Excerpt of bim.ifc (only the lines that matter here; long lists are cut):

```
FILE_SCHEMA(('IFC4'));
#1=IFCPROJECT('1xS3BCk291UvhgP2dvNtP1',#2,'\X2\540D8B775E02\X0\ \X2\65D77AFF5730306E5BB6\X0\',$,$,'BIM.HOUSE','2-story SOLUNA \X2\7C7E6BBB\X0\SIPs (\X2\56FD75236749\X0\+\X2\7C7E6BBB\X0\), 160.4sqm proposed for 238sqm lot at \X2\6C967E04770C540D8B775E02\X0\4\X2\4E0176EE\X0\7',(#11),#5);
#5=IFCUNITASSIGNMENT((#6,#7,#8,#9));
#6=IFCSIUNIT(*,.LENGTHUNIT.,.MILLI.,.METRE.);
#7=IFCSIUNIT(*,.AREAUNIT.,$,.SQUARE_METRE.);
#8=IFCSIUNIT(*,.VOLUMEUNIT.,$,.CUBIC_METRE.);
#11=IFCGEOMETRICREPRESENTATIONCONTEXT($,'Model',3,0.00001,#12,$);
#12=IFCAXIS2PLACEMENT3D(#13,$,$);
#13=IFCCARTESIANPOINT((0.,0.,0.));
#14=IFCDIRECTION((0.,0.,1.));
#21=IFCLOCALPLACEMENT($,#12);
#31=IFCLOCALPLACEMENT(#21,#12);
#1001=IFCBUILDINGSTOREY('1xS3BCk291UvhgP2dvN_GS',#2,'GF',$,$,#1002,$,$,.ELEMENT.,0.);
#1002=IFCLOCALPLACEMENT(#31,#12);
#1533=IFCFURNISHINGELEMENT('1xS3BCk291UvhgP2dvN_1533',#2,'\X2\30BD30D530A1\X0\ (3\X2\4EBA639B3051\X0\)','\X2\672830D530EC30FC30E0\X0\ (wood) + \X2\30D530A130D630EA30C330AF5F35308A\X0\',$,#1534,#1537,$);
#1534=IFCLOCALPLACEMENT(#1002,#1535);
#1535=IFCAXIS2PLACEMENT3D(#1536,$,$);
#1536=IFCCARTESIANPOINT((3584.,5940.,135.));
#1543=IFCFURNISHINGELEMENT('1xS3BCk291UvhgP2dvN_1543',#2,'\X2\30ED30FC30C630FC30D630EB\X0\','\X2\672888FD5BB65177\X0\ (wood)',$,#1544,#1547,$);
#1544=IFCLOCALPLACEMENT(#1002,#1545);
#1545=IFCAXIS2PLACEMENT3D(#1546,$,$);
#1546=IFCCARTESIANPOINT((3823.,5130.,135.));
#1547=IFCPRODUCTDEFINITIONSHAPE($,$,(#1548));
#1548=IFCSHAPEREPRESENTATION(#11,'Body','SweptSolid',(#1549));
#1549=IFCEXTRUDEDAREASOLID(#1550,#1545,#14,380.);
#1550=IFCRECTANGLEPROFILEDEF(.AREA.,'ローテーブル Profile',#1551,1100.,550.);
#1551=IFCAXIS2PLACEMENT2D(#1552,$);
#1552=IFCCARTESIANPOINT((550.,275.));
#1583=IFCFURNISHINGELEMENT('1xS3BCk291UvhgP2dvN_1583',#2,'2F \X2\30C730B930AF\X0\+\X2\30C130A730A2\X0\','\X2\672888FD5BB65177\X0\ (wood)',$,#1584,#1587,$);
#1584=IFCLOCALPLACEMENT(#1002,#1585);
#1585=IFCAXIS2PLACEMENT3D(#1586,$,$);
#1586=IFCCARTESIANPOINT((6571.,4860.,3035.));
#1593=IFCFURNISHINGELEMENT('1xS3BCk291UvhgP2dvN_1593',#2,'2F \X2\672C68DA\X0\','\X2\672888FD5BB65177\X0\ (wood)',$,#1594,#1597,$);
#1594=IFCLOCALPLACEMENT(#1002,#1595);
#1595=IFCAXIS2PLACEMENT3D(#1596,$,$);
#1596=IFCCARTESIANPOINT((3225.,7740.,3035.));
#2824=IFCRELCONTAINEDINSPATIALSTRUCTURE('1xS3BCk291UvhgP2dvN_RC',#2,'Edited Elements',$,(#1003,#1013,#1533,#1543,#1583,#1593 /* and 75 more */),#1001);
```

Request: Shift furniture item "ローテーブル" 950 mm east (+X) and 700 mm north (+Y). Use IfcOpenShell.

```python
import ifcopenshell
import ifcopenshell.api.geometry
import ifcopenshell.util.placement
import ifcopenshell.util.unit

model = ifcopenshell.open("bim.ifc")
unit_scale = ifcopenshell.util.unit.calculate_unit_scale(model)

item = model.by_guid("1xS3BCk291UvhgP2dvN_1543")
matrix = ifcopenshell.util.placement.get_local_placement(item.ObjectPlacement)
matrix[0, 3] += 0.95 / unit_scale
matrix[1, 3] += 0.7 / unit_scale
ifcopenshell.api.geometry.edit_object_placement(model, product=item, matrix=matrix, is_si=False)

print(ifcopenshell.util.placement.get_local_placement(item.ObjectPlacement).round(3) + 0.0)

model.write("bim_v2.ifc")
```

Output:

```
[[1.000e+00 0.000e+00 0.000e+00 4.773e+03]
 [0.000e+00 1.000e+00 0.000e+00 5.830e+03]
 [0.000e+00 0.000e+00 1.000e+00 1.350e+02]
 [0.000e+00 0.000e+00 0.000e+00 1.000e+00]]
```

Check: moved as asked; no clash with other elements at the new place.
